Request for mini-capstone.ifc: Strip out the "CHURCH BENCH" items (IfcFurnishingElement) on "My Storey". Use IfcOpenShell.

First a look at what the model holds.

```python
import ifcopenshell
import ifcopenshell.util.element

model = ifcopenshell.open("mini-capstone.ifc")
print(model.schema)
storey = next(s for s in model.by_type("IfcBuildingStorey") if s.Name == "My Storey")
furniture = [e for e in ifcopenshell.util.element.get_decomposition(storey) if e.is_a("IfcFurnishingElement")]
seen = {}
for e in furniture:
    element_type = ifcopenshell.util.element.get_type(e)
    name = element_type.Name if element_type not in (None, e) else None
    seen[name] = seen.get(name, 0) + 1
for name, count in sorted(seen.items(), key=str):
    print(count, "x", name)
```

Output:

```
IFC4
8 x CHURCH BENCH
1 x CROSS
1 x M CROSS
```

```python
import ifcopenshell
import ifcopenshell.api.root
import ifcopenshell.util.element

model = ifcopenshell.open("mini-capstone.ifc")

storey = next(s for s in model.by_type("IfcBuildingStorey") if s.Name == "My Storey")
furniture = [e for e in ifcopenshell.util.element.get_decomposition(storey) if e.is_a("IfcFurnishingElement")]
targets = [e for e in furniture if (t := ifcopenshell.util.element.get_type(e)) not in (None, e) and t.Name == "CHURCH BENCH"]

for e in targets:
    ifcopenshell.api.root.remove_product(model, product=e)
print(len(targets), "removed")

model.write("mini-capstone_edited.ifc")
```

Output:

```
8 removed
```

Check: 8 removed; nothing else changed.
